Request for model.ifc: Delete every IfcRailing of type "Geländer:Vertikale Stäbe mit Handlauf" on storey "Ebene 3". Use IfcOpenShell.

First a look at what the model holds.

```python
import ifcopenshell
import ifcopenshell.util.element

model = ifcopenshell.open("model.ifc")
print(model.schema)
storey = next(s for s in model.by_type("IfcBuildingStorey") if s.Name == "Ebene 3")
railings = [e for e in ifcopenshell.util.element.get_decomposition(storey) if e.is_a("IfcRailing")]
seen = {}
for e in railings:
    element_type = ifcopenshell.util.element.get_type(e)
    name = element_type.Name if element_type not in (None, e) else None
    seen[name] = seen.get(name, 0) + 1
for name, count in sorted(seen.items(), key=str):
    print(count, "x", name)
```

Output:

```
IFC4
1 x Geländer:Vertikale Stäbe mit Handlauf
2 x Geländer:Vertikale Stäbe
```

```python
import ifcopenshell
import ifcopenshell.api.root
import ifcopenshell.util.element

model = ifcopenshell.open("model.ifc")

storey = next(s for s in model.by_type("IfcBuildingStorey") if s.Name == "Ebene 3")
railings = [e for e in ifcopenshell.util.element.get_decomposition(storey) if e.is_a("IfcRailing")]
targets = [e for e in railings if (t := ifcopenshell.util.element.get_type(e)) not in (None, e) and t.Name == "Geländer:Vertikale Stäbe mit Handlauf"]

for e in targets:
    ifcopenshell.api.root.remove_product(model, product=e)
print(len(targets), "removed")

model.write("model_rev.ifc")
```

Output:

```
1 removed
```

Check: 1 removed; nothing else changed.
